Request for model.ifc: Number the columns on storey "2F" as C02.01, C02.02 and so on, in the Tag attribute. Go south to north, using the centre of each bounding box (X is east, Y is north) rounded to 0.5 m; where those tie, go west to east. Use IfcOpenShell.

First a look at what the model holds.

```python
import ifcopenshell
import ifcopenshell.util.element
import ifcopenshell.util.placement

model = ifcopenshell.open("model.ifc")
print(model.schema)
storey = next(s for s in model.by_type("IfcBuildingStorey") if s.Name == "2F")
columns = [e for e in ifcopenshell.util.element.get_decomposition(storey) if e.is_a("IfcColumn")]
for e in sorted(columns, key=lambda e: e.id()):
    origin = ifcopenshell.util.placement.get_local_placement(e.ObjectPlacement)[:3, 3]
    print(e.id(), e.Tag, e.Name, origin.round(2) + 0.0, sep=" | ")
```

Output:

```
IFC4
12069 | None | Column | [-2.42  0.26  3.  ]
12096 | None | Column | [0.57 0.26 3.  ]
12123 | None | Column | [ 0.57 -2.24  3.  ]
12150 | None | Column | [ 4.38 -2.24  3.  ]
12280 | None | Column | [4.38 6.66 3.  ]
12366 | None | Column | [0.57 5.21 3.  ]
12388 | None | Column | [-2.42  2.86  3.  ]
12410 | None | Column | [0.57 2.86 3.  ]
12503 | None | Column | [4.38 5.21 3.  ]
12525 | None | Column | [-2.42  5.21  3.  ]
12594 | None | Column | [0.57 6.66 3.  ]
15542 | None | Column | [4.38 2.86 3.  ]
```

```python
import ifcopenshell
import ifcopenshell.geom
import ifcopenshell.util.element
import ifcopenshell.util.shape

model = ifcopenshell.open("model.ifc")
settings = ifcopenshell.geom.settings()
settings.set("use-world-coords", True)


def centre(element):
    shape = ifcopenshell.geom.create_shape(settings, element)
    return ifcopenshell.util.shape.get_bbox_centroid(shape.geometry)


storey = next(s for s in model.by_type("IfcBuildingStorey") if s.Name == "2F")
columns = [e for e in ifcopenshell.util.element.get_decomposition(storey) if e.is_a("IfcColumn")]

# Insertion points can sit at a corner or the storey origin, so sort by the geometry (in metres).
centres = {e: centre(e) for e in columns}
columns.sort(key=lambda e: (round(centres[e][1] / 0.5), centres[e][0]))

for i, e in enumerate(columns, start=1):
    number = f"C02.{i:02d}"
    e.Tag = number
    print(e.id(), number)

model.write("model_v2.ifc")
```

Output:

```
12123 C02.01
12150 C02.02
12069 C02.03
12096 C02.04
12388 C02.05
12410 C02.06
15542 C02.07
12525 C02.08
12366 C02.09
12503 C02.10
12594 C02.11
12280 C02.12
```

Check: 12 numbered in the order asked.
